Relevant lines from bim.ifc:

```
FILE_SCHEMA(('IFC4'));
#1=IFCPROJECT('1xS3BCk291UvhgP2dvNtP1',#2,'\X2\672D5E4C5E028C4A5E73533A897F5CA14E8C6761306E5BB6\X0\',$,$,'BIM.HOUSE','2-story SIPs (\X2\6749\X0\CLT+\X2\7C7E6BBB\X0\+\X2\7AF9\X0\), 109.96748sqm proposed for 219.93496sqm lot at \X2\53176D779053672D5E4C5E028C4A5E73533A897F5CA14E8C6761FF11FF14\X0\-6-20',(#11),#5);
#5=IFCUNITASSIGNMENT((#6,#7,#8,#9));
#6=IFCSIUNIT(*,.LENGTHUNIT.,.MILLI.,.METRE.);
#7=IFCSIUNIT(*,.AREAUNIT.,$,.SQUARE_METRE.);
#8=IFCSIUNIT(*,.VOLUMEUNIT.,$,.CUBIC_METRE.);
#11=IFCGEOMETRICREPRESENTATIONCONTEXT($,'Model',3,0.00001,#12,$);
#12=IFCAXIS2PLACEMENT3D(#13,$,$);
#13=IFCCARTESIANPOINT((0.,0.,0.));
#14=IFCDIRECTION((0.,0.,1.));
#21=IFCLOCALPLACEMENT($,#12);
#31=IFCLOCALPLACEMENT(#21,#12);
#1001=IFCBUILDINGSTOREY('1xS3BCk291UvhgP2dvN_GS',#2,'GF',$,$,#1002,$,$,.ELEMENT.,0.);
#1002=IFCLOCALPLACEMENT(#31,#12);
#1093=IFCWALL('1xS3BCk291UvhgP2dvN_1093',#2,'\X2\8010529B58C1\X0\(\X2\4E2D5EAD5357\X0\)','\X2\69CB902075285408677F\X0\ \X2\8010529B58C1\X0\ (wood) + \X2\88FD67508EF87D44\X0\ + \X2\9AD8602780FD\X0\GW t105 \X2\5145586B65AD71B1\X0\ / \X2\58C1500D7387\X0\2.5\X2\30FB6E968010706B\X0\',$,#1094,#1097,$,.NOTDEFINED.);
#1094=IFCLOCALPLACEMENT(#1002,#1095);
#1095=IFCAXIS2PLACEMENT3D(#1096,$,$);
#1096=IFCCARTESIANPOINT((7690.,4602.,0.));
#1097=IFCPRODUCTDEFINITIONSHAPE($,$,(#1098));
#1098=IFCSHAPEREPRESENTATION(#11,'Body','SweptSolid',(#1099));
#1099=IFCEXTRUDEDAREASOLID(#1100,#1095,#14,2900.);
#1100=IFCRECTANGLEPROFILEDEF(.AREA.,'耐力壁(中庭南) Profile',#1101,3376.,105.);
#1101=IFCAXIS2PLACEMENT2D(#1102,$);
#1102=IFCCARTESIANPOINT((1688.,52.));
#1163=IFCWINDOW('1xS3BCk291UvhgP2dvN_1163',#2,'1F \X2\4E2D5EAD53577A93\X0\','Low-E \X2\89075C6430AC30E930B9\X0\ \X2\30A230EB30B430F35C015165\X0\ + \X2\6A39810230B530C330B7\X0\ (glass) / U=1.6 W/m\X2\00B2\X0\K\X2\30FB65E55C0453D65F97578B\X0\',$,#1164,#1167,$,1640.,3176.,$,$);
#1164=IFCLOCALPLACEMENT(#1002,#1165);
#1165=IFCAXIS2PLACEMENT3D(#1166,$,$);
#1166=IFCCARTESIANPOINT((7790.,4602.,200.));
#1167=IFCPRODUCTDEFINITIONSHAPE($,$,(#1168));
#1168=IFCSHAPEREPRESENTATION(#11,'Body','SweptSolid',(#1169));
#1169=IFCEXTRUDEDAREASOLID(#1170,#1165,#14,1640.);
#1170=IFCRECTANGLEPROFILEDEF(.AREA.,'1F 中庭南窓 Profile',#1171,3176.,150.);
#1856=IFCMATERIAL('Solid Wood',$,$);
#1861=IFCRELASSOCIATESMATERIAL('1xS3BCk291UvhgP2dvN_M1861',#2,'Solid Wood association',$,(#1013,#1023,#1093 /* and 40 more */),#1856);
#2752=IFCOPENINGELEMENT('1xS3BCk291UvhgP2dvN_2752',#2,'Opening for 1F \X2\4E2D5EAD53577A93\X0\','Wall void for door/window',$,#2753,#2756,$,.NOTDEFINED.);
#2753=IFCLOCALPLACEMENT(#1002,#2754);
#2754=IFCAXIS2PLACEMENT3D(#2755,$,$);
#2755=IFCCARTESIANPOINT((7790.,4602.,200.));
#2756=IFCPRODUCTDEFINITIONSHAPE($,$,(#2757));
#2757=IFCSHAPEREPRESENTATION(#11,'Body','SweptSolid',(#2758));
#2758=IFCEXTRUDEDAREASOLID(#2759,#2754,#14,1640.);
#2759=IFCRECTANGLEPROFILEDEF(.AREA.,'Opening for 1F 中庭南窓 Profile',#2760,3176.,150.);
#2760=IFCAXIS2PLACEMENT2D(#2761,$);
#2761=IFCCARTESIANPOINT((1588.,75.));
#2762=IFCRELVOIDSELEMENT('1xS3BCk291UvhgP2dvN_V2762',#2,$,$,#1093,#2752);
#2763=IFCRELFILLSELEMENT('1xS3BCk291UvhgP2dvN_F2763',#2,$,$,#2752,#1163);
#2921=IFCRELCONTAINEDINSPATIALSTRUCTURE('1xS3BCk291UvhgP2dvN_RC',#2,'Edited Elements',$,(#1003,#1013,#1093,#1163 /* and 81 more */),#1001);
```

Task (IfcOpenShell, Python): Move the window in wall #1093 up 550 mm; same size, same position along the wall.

```python
import numpy as np
import ifcopenshell
import ifcopenshell.api.geometry
import ifcopenshell.util.placement
import ifcopenshell.util.unit

model = ifcopenshell.open("bim.ifc")
unit_scale = ifcopenshell.util.unit.calculate_unit_scale(model)

window = model.by_guid("1xS3BCk291UvhgP2dvN_1163")
opening = window.FillsVoids[0].RelatingOpeningElement
dz = 550.0

shift = np.array([0.0, 0.0, dz])
# The window is not placed relative to its opening, so move both.
for product in (opening, window):
    matrix = ifcopenshell.util.placement.get_local_placement(product.ObjectPlacement)
    matrix[:3, 3] += shift
    ifcopenshell.api.geometry.edit_object_placement(model, product=product, matrix=matrix, is_si=False)

print(f"moved by {dz * unit_scale:+.3f} m")

model.write("bim_edited.ifc")
```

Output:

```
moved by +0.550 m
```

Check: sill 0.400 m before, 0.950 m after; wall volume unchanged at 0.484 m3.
